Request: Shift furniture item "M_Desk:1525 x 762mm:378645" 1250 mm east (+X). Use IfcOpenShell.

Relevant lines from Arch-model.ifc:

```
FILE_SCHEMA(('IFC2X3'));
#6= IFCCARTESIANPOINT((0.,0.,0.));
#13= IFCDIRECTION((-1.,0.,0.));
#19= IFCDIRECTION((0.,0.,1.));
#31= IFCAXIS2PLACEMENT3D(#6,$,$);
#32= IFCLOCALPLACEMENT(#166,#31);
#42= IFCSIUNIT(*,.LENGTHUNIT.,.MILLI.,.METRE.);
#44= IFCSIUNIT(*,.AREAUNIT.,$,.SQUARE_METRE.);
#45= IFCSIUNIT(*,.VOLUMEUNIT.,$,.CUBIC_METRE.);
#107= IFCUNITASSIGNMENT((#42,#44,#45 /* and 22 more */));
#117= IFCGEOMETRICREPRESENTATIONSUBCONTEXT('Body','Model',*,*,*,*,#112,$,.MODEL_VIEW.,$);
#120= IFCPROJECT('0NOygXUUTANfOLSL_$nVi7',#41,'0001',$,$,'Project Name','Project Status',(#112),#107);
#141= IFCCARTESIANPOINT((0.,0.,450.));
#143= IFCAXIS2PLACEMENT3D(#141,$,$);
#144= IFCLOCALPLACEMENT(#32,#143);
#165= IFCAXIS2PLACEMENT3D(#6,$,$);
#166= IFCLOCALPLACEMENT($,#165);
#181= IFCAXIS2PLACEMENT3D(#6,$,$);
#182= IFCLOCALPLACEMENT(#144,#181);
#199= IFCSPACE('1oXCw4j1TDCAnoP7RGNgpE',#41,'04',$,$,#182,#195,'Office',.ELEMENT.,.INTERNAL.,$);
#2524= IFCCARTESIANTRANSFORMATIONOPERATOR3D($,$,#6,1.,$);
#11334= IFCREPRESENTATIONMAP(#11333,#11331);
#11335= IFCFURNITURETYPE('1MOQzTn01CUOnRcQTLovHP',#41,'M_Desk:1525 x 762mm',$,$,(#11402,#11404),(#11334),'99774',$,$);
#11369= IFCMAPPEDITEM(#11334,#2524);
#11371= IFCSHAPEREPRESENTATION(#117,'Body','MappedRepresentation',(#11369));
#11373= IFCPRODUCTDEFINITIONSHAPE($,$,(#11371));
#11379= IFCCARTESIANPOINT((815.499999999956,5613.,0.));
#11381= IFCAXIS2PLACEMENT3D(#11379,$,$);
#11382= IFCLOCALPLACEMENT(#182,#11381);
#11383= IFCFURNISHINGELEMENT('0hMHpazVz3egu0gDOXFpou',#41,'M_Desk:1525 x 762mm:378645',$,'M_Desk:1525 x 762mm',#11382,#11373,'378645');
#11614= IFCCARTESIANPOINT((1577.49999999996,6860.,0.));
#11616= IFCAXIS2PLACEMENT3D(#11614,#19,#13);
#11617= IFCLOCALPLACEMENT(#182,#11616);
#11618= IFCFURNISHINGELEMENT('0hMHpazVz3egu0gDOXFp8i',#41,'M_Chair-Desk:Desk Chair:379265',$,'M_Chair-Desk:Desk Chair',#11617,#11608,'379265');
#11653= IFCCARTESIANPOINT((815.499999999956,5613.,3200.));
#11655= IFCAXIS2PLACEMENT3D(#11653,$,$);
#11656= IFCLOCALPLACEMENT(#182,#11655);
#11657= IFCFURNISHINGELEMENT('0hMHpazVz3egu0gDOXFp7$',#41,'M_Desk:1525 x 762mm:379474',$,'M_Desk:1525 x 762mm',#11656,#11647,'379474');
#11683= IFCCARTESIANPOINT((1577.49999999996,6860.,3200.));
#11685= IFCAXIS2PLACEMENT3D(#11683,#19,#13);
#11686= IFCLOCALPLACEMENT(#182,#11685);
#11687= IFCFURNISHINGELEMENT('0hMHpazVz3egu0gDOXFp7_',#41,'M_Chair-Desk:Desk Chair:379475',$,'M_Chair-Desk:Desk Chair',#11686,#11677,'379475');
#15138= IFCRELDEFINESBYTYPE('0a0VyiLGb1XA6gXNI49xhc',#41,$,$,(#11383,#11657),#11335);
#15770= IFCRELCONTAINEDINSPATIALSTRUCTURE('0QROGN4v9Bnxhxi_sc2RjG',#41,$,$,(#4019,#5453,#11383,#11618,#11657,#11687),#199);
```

```python
import ifcopenshell
import ifcopenshell.api.geometry
import ifcopenshell.util.placement
import ifcopenshell.util.unit

model = ifcopenshell.open("Arch-model.ifc")
unit_scale = ifcopenshell.util.unit.calculate_unit_scale(model)

item = model.by_guid("0hMHpazVz3egu0gDOXFpou")
matrix = ifcopenshell.util.placement.get_local_placement(item.ObjectPlacement)
matrix[0, 3] += 1.25 / unit_scale
ifcopenshell.api.geometry.edit_object_placement(model, product=item, matrix=matrix, is_si=False)

print(ifcopenshell.util.placement.get_local_placement(item.ObjectPlacement).round(3) + 0.0)

model.write("Arch-model_edited.ifc")
```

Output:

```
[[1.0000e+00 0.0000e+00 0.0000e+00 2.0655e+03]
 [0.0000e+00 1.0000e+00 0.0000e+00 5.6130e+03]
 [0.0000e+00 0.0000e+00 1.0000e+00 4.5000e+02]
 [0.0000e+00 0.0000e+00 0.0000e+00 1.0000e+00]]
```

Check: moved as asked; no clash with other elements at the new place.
